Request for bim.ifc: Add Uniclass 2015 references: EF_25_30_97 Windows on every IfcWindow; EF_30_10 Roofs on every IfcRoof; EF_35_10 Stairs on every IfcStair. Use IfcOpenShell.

First a look at what the model holds.

```python
import ifcopenshell

model = ifcopenshell.open("bim.ifc")
print(model.schema)
print("classifications:", [c.Name for c in model.by_type("IfcClassification")])
for ifc_class in ("IfcDoor", "IfcRoof", "IfcStair", "IfcWall", "IfcWindow"):
    print(ifc_class, len(model.by_type(ifc_class)))
```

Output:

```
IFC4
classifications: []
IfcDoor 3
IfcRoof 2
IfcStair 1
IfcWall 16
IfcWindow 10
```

```python
import ifcopenshell
import ifcopenshell.api.classification

model = ifcopenshell.open("bim.ifc")

system = ifcopenshell.api.classification.add_classification(model, classification="Uniclass 2015")

codes = {
    "IfcWindow": ("EF_25_30_97", "Windows"),
    "IfcRoof": ("EF_30_10", "Roofs"),
    "IfcStair": ("EF_35_10", "Stairs"),
}
for ifc_class, (code, name) in codes.items():
    products = model.by_type(ifc_class)
    ifcopenshell.api.classification.add_reference(
        model, products=products, classification=system, identification=code, name=name
    )
    print(code, len(products))

model.write("bim_edited.ifc")
```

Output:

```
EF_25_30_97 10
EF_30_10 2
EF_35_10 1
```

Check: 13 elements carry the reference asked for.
